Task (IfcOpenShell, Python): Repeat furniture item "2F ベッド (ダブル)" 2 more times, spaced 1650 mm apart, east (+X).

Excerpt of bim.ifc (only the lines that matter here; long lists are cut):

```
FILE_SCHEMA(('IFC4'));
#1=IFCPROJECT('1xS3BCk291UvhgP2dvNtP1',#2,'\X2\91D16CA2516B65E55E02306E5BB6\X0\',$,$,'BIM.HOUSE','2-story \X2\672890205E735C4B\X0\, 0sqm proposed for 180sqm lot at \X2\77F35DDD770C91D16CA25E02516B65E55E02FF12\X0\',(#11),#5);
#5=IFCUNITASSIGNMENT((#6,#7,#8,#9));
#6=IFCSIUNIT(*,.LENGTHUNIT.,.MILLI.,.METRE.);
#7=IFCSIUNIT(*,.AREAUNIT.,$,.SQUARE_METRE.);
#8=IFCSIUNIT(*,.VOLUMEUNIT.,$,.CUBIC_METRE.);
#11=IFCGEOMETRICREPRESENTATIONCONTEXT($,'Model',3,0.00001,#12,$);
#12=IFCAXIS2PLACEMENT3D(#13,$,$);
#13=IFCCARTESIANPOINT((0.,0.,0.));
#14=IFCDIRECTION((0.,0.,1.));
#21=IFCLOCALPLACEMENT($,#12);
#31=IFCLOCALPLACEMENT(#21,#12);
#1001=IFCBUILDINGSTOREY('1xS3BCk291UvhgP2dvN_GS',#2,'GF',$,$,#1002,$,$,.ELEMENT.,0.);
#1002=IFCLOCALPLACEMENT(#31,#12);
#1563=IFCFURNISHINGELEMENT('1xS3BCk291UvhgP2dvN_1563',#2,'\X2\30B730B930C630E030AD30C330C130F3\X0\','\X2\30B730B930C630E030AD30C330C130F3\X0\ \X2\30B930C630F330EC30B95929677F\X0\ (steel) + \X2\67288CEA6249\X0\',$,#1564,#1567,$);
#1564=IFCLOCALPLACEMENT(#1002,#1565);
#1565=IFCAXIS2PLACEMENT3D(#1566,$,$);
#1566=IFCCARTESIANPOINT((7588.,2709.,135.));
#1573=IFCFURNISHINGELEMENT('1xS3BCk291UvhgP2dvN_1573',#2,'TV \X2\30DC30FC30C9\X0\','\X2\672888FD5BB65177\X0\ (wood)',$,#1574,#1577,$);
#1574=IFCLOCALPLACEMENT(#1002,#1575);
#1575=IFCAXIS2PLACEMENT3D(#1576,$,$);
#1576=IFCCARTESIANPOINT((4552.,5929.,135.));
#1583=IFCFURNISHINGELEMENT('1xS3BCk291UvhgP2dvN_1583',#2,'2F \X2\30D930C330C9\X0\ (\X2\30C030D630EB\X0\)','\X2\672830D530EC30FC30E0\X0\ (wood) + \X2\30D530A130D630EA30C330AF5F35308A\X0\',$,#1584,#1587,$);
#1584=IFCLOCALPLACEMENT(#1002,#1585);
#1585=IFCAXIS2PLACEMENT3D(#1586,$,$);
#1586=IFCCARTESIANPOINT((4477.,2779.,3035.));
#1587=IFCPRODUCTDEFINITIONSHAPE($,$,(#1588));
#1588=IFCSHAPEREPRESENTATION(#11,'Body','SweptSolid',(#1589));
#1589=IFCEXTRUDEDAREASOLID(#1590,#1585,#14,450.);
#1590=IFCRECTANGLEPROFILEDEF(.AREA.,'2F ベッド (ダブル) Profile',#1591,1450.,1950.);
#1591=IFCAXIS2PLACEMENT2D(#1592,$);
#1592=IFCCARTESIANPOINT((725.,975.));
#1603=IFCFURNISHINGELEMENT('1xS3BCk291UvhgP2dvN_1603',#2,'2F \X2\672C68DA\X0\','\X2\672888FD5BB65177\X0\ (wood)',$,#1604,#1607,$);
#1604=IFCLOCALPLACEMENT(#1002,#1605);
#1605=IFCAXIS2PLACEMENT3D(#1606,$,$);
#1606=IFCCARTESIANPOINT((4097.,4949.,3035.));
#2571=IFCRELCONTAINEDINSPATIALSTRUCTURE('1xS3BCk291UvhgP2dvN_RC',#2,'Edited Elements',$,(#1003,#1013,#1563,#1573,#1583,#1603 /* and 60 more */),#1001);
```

```python
import numpy as np
import ifcopenshell
import ifcopenshell.api.geometry
import ifcopenshell.api.root
import ifcopenshell.util.element
import ifcopenshell.util.placement
import ifcopenshell.util.unit

model = ifcopenshell.open("bim.ifc")
unit_scale = ifcopenshell.util.unit.calculate_unit_scale(model)


def reuse_history(source, copy):
    """copy_class also copies each property set's owner history, people and application; keep the originals."""
    for rel in copy.IsDefinedBy:
        if rel.is_a("IfcRelDefinesByProperties") and (history := rel.RelatingPropertyDefinition.OwnerHistory):
            rel.RelatingPropertyDefinition.OwnerHistory = source.OwnerHistory
            ifcopenshell.util.element.remove_deep2(model, history)


source = model.by_id(1583)
base = ifcopenshell.util.placement.get_local_placement(source.ObjectPlacement)
step = np.array([1.0, 0.0, 0.0]) * 1.65 / unit_scale

for i in range(1, 3):
    copy = ifcopenshell.api.root.copy_class(model, product=source)
    copy.Representation = ifcopenshell.util.element.copy_deep(
        model, source.Representation, exclude=["IfcGeometricRepresentationContext", "IfcRepresentationMap"]
    )
    reuse_history(source, copy)
    matrix = base.copy()
    matrix[:3, 3] += i * step
    print("added at", matrix[:3, 3].round(3) + 0.0)
    ifcopenshell.api.geometry.edit_object_placement(model, product=copy, matrix=matrix, is_si=False)

model.write("bim_v2.ifc")
```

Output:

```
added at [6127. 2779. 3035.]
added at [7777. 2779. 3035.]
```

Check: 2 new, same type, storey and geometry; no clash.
